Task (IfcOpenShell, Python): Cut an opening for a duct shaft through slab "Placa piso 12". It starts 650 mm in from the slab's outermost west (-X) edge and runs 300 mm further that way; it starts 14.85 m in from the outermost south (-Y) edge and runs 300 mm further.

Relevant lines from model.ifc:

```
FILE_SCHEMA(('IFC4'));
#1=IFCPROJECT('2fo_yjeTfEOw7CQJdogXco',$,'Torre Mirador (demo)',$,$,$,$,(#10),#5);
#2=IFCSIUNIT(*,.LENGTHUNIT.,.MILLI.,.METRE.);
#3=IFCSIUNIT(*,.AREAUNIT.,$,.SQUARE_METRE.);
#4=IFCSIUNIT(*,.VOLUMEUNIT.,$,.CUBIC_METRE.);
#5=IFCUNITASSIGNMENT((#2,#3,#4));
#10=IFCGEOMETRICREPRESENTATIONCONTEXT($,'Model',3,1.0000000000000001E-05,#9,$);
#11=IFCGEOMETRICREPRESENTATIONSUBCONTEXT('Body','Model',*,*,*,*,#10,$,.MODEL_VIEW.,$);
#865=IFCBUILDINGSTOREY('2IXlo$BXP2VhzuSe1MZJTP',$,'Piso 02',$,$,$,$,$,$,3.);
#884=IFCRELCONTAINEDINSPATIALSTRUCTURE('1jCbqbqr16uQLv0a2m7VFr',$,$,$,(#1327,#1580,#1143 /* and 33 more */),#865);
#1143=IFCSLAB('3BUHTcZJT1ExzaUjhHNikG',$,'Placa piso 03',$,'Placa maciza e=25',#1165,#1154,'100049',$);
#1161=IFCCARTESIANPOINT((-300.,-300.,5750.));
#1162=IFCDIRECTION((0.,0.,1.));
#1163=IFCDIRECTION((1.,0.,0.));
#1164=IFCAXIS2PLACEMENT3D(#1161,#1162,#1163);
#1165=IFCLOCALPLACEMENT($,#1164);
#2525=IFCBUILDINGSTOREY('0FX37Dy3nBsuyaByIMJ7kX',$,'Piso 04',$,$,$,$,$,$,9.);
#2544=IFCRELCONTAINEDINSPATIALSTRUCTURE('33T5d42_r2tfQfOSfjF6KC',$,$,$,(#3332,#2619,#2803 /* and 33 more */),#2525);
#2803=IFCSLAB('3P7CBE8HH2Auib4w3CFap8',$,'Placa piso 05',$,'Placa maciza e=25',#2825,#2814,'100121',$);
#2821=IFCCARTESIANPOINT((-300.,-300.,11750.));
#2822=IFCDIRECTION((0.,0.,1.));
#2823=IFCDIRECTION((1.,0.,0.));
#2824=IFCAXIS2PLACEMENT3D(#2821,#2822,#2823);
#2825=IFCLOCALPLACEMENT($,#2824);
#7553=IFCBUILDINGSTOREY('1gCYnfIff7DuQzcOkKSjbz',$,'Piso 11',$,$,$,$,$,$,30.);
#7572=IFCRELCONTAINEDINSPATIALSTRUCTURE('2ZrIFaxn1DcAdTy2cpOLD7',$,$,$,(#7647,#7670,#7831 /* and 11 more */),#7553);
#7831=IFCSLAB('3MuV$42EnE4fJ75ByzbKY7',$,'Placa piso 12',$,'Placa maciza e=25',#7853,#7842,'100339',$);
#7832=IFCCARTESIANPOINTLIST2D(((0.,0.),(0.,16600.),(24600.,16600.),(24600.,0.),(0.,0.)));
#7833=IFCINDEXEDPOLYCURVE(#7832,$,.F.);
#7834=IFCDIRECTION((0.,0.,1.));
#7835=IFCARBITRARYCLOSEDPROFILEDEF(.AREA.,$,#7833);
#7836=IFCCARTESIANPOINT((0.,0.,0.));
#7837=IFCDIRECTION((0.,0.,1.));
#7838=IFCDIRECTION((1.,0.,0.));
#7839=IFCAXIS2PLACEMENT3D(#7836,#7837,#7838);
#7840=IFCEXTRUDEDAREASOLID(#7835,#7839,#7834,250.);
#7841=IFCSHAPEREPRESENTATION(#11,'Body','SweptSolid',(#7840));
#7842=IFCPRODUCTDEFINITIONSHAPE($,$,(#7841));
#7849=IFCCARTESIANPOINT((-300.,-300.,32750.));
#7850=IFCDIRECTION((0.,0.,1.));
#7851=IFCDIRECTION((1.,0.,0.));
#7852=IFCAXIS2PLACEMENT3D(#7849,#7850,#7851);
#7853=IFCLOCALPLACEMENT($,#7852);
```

```python
import numpy as np
import ifcopenshell
import ifcopenshell.api.feature
import ifcopenshell.api.geometry
import ifcopenshell.api.root
import ifcopenshell.geom
import ifcopenshell.util.placement
import ifcopenshell.util.representation
import ifcopenshell.util.shape
import ifcopenshell.util.unit

model = ifcopenshell.open("model.ifc")
unit_scale = ifcopenshell.util.unit.calculate_unit_scale(model)
settings = ifcopenshell.geom.settings()


def volume(element):
    """Net volume in cubic metres, openings subtracted."""
    shape = ifcopenshell.geom.create_shape(settings, element)
    return ifcopenshell.util.shape.get_volume(shape.geometry)


slab = model.by_guid("3MuV$42EnE4fJ75ByzbKY7")
before = volume(slab)

# Extent in the slab's own axes, in metres. The edges named are its -X and -Y sides.
slab_shape = ifcopenshell.geom.create_shape(settings, slab)
vertices = ifcopenshell.util.shape.get_vertices(slab_shape.geometry)
x_min, y_min, bottom = vertices.min(axis=0)
top = vertices[:, 2].max()

opening = ifcopenshell.api.root.create_entity(model, ifc_class="IfcOpeningElement", name="Duct shaft opening", predefined_type="OPENING")
context = ifcopenshell.util.representation.get_context(model, "Model", "Body", "MODEL_VIEW")
width, depth = 0.3, 0.3
outline = [(0.0, 0.0), (width, 0.0), (width, depth), (0.0, depth), (0.0, 0.0)]
# Overshoot both faces by 50 mm so the cut is clean.
shape = ifcopenshell.api.geometry.add_slab_representation(
    model, context=context, depth=top - bottom + 0.1, polyline=outline
)
ifcopenshell.api.geometry.assign_representation(model, product=opening, representation=shape)

matrix = ifcopenshell.util.placement.get_local_placement(slab.ObjectPlacement)
matrix[:, 3] = matrix @ np.append(np.array([x_min + 0.65, y_min + 14.85, bottom - 0.05]) / unit_scale, 1.0)
ifcopenshell.api.geometry.edit_object_placement(model, product=opening, matrix=matrix, is_si=False)
ifcopenshell.api.feature.add_feature(model, feature=opening, element=slab)

after = volume(slab)

print(f"slab volume {before:.3f} -> {after:.3f} m3")

model.write("model_edited.ifc")
```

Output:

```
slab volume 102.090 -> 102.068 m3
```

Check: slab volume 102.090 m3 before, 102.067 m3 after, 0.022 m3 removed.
